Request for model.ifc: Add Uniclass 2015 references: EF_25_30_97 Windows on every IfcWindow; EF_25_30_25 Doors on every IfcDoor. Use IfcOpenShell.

First a look at what the model holds.

```python
import ifcopenshell

model = ifcopenshell.open("model.ifc")
print(model.schema)
print("classifications:", [c.Name for c in model.by_type("IfcClassification")])
for ifc_class in ("IfcDoor", "IfcRoof", "IfcStair", "IfcWall", "IfcWindow"):
    print(ifc_class, len(model.by_type(ifc_class)))
```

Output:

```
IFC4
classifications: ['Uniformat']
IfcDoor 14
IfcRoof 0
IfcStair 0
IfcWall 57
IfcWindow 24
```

```python
import ifcopenshell
import ifcopenshell.api.classification

model = ifcopenshell.open("model.ifc")

system = ifcopenshell.api.classification.add_classification(model, classification="Uniclass 2015")

codes = {
    "IfcWindow": ("EF_25_30_97", "Windows"),
    "IfcDoor": ("EF_25_30_25", "Doors"),
}
for ifc_class, (code, name) in codes.items():
    products = model.by_type(ifc_class)
    ifcopenshell.api.classification.add_reference(
        model, products=products, classification=system, identification=code, name=name
    )
    print(code, len(products))

model.write("model_rev.ifc")
```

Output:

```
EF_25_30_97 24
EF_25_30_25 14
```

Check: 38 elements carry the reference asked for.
